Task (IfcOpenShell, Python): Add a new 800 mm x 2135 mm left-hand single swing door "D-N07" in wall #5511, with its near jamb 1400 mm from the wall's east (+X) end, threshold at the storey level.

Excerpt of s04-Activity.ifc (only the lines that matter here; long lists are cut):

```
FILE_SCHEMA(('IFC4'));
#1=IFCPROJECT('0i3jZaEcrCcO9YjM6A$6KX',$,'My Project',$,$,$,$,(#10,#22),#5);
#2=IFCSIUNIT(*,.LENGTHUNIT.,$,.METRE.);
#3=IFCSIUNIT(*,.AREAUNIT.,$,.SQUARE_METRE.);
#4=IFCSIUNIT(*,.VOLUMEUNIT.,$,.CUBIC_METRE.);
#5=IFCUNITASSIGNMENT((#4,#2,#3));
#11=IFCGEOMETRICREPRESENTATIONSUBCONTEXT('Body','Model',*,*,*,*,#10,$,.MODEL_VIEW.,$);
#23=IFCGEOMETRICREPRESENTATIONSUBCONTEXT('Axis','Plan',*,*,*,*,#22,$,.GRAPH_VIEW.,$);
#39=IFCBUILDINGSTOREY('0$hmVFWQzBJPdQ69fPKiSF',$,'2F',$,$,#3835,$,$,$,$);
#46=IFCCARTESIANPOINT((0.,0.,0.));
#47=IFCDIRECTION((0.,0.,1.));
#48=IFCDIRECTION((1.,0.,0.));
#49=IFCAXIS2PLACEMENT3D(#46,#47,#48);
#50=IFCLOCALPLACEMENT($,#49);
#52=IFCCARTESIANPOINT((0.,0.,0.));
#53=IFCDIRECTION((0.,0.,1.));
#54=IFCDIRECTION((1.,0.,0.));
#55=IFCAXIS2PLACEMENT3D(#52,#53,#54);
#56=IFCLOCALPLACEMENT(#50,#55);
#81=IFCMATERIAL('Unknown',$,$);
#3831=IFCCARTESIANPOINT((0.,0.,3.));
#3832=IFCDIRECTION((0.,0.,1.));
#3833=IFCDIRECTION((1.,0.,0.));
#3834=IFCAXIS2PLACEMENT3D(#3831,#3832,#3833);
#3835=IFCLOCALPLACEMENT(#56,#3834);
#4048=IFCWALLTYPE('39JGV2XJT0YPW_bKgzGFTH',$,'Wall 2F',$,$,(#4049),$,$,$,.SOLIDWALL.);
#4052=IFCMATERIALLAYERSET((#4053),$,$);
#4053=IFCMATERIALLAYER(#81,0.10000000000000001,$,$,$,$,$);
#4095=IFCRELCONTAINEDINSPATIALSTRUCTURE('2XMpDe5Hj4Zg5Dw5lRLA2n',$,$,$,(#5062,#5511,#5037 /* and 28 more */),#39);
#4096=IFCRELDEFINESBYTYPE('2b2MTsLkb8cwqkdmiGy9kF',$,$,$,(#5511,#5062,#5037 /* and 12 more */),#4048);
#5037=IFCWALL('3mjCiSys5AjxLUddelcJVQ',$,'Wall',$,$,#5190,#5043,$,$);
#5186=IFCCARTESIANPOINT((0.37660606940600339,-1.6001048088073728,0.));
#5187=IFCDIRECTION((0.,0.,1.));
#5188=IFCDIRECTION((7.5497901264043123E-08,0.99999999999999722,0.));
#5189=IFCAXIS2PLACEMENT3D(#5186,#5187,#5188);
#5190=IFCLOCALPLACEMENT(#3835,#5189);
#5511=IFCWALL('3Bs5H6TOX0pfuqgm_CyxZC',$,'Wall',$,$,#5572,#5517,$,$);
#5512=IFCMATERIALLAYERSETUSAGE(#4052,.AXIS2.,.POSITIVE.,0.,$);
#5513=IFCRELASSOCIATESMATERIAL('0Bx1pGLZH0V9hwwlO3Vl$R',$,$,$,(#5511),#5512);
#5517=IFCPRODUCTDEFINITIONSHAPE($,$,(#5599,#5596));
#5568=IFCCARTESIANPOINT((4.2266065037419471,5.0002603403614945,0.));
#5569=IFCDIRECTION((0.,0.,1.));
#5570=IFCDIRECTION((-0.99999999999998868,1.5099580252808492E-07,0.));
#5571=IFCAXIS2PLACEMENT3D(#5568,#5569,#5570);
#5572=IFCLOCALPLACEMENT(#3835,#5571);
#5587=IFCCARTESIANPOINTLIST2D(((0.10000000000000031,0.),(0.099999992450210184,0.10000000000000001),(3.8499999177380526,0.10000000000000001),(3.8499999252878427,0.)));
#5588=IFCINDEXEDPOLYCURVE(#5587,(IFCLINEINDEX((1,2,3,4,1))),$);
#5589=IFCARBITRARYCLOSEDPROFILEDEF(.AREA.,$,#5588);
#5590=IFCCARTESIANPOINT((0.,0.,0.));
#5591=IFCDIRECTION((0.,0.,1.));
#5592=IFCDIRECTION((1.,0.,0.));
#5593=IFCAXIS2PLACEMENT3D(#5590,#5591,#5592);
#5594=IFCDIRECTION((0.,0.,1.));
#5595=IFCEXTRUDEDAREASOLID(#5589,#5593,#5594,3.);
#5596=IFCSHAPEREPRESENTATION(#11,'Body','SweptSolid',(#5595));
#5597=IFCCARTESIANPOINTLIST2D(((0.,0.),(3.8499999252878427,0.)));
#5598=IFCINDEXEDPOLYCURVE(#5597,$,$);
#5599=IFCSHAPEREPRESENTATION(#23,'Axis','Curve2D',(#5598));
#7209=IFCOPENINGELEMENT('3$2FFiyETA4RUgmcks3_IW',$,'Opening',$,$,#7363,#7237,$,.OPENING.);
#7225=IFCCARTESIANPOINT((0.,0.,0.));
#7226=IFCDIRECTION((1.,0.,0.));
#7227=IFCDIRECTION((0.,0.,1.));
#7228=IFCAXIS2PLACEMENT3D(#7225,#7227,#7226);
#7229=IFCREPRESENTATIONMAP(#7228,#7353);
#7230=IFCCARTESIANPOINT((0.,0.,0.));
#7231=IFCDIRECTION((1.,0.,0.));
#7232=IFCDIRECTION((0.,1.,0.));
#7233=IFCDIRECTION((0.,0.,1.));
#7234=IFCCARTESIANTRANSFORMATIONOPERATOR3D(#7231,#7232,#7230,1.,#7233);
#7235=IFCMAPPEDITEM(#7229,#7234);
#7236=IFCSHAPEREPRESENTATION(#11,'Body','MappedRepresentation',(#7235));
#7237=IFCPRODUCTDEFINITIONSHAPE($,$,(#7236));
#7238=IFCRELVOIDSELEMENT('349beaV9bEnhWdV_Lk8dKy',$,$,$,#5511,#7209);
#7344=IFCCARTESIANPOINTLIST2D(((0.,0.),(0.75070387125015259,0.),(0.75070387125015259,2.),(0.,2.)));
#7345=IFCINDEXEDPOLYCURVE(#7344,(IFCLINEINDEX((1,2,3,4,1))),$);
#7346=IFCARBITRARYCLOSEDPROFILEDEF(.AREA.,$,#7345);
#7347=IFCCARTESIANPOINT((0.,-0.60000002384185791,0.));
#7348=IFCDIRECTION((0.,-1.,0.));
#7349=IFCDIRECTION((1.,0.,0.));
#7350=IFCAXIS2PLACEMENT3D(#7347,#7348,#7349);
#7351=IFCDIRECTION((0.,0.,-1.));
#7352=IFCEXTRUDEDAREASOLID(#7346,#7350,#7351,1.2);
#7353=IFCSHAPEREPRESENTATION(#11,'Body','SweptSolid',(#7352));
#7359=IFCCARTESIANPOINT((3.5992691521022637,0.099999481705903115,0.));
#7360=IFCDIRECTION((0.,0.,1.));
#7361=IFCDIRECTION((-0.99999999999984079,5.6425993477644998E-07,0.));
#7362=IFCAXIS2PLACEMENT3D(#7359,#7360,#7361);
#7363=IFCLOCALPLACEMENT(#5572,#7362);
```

```python
import numpy as np
import ifcopenshell
import ifcopenshell.api.feature
import ifcopenshell.api.geometry
import ifcopenshell.api.root
import ifcopenshell.api.spatial
import ifcopenshell.geom
import ifcopenshell.util.element
import ifcopenshell.util.placement
import ifcopenshell.util.representation
import ifcopenshell.util.shape
import ifcopenshell.util.unit

model = ifcopenshell.open("s04-Activity.ifc")
unit_scale = ifcopenshell.util.unit.calculate_unit_scale(model)
settings = ifcopenshell.geom.settings()


def volume(element):
    """Net volume in cubic metres, openings subtracted."""
    shape = ifcopenshell.geom.create_shape(settings, element)
    return ifcopenshell.util.shape.get_volume(shape.geometry)


wall = model.by_id(5511)
storey = ifcopenshell.util.element.get_container(wall, ifc_class="IfcBuildingStorey")
context = ifcopenshell.util.representation.get_context(model, "Model", "Body", "MODEL_VIEW")
before = volume(wall)

width, height, from_end, sill = 0.8, 2.135, 1.4, 0.0  # metres

# The wall runs along its own X axis, and the end named is its -X end.
wall_shape = ifcopenshell.geom.create_shape(settings, wall)
x, y, z = ifcopenshell.util.shape.get_vertices(wall_shape.geometry).T
start = x.min() + from_end
face, thickness = float(y.min()), float(y.max() - y.min())
wall_matrix = ifcopenshell.util.placement.get_local_placement(wall.ObjectPlacement)
level = ifcopenshell.util.placement.get_local_placement(storey.ObjectPlacement)[2, 3]


def in_wall(x, y):
    """Placement at x, y metres in the wall's axes, at sill height."""
    matrix = wall_matrix.copy()
    matrix[:, 3] = wall_matrix @ np.array([x / unit_scale, y / unit_scale, 0.0, 1.0])
    matrix[2, 3] = level + sill / unit_scale
    return matrix


# Opening: a box that overshoots both wall faces by 50 mm.
opening = ifcopenshell.api.root.create_entity(model, ifc_class="IfcOpeningElement", predefined_type="OPENING")
box = ifcopenshell.api.geometry.add_wall_representation(
    model, context=context, length=width, height=height, thickness=thickness + 0.1
)
ifcopenshell.api.geometry.assign_representation(model, product=opening, representation=box)
ifcopenshell.api.geometry.edit_object_placement(model, product=opening, matrix=in_wall(start, face - 0.05), is_si=False)
ifcopenshell.api.feature.add_feature(model, feature=opening, element=wall)

door = ifcopenshell.api.root.create_entity(model, ifc_class="IfcDoor", name="D-N07", predefined_type="DOOR")
door.OverallWidth, door.OverallHeight = width / unit_scale, height / unit_scale
door.OperationType = "SINGLE_SWING_LEFT"
body = ifcopenshell.api.geometry.add_door_representation(
    model,
    context=context,
    overall_width=door.OverallWidth,
    overall_height=door.OverallHeight,
    operation_type="SINGLE_SWING_LEFT",
    lining_properties={"LiningDepth": thickness / unit_scale, "ThresholdDepth": thickness / unit_scale},
)
ifcopenshell.api.geometry.assign_representation(model, product=door, representation=body)
ifcopenshell.api.spatial.assign_container(model, products=[door], relating_structure=storey)
ifcopenshell.api.feature.add_filling(model, opening=opening, element=door)

# The lining spans the wall, so the door starts at the wall face.
ifcopenshell.api.geometry.edit_object_placement(model, product=door, matrix=in_wall(start, face), is_si=False)

after = volume(wall)

print(f"wall volume {before:.3f} -> {after:.3f} m3")

model.write("s04-Activity_v2.ifc")
```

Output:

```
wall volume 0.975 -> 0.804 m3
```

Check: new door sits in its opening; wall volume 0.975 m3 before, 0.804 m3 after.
